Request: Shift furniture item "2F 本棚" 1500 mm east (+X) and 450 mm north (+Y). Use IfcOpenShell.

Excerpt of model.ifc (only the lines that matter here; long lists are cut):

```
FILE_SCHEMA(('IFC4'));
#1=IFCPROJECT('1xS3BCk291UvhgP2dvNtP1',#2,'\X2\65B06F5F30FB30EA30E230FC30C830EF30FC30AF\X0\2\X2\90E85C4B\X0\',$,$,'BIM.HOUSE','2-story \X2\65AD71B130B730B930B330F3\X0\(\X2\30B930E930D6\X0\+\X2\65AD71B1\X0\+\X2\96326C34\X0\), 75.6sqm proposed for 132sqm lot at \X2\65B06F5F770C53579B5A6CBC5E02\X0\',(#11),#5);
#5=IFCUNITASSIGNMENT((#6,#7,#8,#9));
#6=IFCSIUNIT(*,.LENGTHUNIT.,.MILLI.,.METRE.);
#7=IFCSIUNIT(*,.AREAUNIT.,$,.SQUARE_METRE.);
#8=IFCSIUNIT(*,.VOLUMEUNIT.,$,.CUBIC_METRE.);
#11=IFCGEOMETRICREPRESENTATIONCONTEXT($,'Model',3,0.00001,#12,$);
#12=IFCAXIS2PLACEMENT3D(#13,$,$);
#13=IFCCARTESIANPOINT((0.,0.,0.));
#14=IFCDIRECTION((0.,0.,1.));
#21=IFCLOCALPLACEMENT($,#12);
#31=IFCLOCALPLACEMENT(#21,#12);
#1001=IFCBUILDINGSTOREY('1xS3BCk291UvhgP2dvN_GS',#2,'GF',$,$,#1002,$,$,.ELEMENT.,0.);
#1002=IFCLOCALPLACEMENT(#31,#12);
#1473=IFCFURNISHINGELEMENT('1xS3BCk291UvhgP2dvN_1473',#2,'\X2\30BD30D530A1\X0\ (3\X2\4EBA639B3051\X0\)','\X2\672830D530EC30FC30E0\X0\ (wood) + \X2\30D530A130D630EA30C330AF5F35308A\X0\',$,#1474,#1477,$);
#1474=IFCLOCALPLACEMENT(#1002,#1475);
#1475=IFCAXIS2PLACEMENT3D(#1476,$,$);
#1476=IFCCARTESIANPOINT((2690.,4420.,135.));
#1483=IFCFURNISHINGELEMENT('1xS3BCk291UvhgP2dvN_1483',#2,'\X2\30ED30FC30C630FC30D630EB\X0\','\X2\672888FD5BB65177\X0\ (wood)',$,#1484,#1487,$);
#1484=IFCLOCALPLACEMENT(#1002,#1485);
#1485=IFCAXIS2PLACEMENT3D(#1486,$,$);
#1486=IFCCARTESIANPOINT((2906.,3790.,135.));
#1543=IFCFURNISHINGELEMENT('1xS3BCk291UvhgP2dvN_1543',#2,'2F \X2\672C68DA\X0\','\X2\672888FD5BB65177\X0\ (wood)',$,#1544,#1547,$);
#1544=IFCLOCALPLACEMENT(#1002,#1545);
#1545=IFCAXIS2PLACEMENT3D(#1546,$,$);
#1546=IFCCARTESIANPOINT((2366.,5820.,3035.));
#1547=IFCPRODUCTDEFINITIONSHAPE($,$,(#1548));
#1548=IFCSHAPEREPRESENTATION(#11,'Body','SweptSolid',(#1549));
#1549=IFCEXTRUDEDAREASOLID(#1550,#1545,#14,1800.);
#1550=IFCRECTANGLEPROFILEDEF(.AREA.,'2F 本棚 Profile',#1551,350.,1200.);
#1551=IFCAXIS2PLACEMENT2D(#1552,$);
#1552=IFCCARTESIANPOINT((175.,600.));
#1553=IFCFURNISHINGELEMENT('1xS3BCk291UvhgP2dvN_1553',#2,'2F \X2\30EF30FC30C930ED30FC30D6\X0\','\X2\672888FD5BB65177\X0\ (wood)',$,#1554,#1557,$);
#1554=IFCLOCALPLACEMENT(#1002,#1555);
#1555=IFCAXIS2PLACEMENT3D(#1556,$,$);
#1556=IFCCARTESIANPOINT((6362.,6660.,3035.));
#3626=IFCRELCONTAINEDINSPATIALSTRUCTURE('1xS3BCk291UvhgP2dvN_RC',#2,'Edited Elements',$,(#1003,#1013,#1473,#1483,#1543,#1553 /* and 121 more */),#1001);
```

```python
import ifcopenshell
import ifcopenshell.api.geometry
import ifcopenshell.util.placement
import ifcopenshell.util.unit

model = ifcopenshell.open("model.ifc")
unit_scale = ifcopenshell.util.unit.calculate_unit_scale(model)

item = model.by_id(1543)
matrix = ifcopenshell.util.placement.get_local_placement(item.ObjectPlacement)
matrix[0, 3] += 1.5 / unit_scale
matrix[1, 3] += 0.45 / unit_scale
ifcopenshell.api.geometry.edit_object_placement(model, product=item, matrix=matrix, is_si=False)

print(ifcopenshell.util.placement.get_local_placement(item.ObjectPlacement).round(3) + 0.0)

model.write("model_edited.ifc")
```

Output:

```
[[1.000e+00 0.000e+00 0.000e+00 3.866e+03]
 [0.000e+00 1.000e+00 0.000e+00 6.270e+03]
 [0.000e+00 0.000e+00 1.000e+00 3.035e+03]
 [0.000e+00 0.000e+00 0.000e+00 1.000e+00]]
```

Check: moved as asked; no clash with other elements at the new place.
